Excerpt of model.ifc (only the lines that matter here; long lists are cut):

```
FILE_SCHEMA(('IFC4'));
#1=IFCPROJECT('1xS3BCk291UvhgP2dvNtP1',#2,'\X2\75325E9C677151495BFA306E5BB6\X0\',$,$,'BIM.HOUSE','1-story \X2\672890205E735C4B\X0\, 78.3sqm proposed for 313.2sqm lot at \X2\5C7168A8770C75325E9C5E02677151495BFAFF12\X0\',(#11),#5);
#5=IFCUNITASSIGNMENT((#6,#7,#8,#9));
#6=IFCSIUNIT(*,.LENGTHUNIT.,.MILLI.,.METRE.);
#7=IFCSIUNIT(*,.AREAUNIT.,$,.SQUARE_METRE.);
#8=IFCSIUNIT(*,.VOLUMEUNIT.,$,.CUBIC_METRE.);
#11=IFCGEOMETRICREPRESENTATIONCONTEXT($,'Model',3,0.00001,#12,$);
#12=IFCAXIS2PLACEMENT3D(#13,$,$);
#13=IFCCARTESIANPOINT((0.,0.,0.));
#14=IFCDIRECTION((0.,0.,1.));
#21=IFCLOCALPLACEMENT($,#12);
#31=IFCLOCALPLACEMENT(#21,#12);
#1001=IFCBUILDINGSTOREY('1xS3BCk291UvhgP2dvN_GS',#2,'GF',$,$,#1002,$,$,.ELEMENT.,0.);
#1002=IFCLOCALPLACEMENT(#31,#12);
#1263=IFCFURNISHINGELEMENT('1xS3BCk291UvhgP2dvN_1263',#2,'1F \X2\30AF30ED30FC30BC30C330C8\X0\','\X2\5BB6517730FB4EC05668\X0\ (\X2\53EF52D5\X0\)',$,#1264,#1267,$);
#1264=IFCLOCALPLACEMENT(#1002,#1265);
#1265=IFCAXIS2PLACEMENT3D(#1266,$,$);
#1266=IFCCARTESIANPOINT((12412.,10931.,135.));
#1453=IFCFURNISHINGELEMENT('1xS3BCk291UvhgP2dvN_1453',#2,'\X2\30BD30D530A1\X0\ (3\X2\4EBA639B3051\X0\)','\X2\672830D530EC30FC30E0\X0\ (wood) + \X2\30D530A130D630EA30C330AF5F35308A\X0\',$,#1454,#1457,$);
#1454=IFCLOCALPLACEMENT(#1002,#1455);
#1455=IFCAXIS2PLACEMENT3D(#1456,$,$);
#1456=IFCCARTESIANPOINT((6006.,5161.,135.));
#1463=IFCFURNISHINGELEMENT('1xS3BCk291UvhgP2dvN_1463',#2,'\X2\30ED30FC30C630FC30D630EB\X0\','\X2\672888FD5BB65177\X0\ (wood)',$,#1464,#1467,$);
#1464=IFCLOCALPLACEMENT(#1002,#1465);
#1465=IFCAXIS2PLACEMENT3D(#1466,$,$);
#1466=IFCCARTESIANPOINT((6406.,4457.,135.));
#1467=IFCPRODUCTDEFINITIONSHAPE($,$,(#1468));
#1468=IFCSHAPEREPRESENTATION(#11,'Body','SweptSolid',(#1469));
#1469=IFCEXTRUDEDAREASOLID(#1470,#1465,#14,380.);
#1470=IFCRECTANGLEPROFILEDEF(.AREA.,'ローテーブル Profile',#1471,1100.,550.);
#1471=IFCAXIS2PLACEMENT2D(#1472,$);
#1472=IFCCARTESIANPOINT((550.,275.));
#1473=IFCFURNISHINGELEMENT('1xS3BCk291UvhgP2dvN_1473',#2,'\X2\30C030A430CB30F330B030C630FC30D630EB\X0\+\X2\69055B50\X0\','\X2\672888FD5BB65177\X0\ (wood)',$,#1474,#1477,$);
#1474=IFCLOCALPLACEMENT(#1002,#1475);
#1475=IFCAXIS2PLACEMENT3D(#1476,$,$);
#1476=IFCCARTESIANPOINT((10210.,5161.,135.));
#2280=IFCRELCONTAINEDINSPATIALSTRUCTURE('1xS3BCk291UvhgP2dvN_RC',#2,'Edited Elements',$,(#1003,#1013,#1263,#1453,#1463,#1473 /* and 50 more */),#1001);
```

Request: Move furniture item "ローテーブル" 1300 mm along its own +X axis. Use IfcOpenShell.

```python
import ifcopenshell
import ifcopenshell.api.geometry
import ifcopenshell.util.placement
import ifcopenshell.util.unit

model = ifcopenshell.open("model.ifc")
unit_scale = ifcopenshell.util.unit.calculate_unit_scale(model)

item = model.by_guid("1xS3BCk291UvhgP2dvN_1463")
matrix = ifcopenshell.util.placement.get_local_placement(item.ObjectPlacement)
matrix[:3, 3] += matrix[:3, 0] * 1.3 / unit_scale
ifcopenshell.api.geometry.edit_object_placement(model, product=item, matrix=matrix, is_si=False)

print(ifcopenshell.util.placement.get_local_placement(item.ObjectPlacement).round(3) + 0.0)

model.write("model-out.ifc")
```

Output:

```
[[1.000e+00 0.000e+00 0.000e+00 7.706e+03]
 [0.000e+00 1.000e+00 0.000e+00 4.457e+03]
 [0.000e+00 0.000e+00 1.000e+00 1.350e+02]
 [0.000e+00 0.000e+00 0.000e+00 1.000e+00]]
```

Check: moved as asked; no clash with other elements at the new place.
